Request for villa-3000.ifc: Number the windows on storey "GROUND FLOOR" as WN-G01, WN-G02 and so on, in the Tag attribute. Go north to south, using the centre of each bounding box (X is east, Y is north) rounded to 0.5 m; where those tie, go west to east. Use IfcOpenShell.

First a look at what the model holds.

```python
import ifcopenshell
import ifcopenshell.util.element
import ifcopenshell.util.placement

model = ifcopenshell.open("villa-3000.ifc")
print(model.schema)
storey = next(s for s in model.by_type("IfcBuildingStorey") if s.Name == "GROUND FLOOR")
windows = [e for e in ifcopenshell.util.element.get_decomposition(storey) if e.is_a("IfcWindow")]
for e in sorted(windows, key=lambda e: e.id()):
    origin = ifcopenshell.util.placement.get_local_placement(e.ObjectPlacement)[:3, 3]
    print(e.id(), e.Tag, e.Name, origin.round(2) + 0.0, sep=" | ")
```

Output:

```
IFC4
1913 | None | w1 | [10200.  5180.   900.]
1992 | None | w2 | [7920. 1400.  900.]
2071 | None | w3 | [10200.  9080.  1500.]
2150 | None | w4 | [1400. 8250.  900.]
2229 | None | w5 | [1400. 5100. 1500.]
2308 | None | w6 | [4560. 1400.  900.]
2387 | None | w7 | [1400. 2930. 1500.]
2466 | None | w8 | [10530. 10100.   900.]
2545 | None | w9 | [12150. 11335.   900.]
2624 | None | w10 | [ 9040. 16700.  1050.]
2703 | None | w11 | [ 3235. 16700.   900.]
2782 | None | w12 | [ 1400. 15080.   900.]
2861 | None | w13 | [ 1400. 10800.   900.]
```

```python
import ifcopenshell
import ifcopenshell.geom
import ifcopenshell.util.element
import ifcopenshell.util.shape

model = ifcopenshell.open("villa-3000.ifc")
settings = ifcopenshell.geom.settings()
settings.set("use-world-coords", True)


def centre(element):
    shape = ifcopenshell.geom.create_shape(settings, element)
    return ifcopenshell.util.shape.get_bbox_centroid(shape.geometry)


storey = next(s for s in model.by_type("IfcBuildingStorey") if s.Name == "GROUND FLOOR")
windows = [e for e in ifcopenshell.util.element.get_decomposition(storey) if e.is_a("IfcWindow")]

# Insertion points can sit at a corner or the storey origin, so sort by the geometry (in metres).
centres = {e: centre(e) for e in windows}
windows.sort(key=lambda e: (-round(centres[e][1] / 0.5), centres[e][0]))

for i, e in enumerate(windows, start=1):
    number = f"WN-G{i:02d}"
    e.Tag = number
    print(e.id(), number)

model.write("villa-3000_v2.ifc")
```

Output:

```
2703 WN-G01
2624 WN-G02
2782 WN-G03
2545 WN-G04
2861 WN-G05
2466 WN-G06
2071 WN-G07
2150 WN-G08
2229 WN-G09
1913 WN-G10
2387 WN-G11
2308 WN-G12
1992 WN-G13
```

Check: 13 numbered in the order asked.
